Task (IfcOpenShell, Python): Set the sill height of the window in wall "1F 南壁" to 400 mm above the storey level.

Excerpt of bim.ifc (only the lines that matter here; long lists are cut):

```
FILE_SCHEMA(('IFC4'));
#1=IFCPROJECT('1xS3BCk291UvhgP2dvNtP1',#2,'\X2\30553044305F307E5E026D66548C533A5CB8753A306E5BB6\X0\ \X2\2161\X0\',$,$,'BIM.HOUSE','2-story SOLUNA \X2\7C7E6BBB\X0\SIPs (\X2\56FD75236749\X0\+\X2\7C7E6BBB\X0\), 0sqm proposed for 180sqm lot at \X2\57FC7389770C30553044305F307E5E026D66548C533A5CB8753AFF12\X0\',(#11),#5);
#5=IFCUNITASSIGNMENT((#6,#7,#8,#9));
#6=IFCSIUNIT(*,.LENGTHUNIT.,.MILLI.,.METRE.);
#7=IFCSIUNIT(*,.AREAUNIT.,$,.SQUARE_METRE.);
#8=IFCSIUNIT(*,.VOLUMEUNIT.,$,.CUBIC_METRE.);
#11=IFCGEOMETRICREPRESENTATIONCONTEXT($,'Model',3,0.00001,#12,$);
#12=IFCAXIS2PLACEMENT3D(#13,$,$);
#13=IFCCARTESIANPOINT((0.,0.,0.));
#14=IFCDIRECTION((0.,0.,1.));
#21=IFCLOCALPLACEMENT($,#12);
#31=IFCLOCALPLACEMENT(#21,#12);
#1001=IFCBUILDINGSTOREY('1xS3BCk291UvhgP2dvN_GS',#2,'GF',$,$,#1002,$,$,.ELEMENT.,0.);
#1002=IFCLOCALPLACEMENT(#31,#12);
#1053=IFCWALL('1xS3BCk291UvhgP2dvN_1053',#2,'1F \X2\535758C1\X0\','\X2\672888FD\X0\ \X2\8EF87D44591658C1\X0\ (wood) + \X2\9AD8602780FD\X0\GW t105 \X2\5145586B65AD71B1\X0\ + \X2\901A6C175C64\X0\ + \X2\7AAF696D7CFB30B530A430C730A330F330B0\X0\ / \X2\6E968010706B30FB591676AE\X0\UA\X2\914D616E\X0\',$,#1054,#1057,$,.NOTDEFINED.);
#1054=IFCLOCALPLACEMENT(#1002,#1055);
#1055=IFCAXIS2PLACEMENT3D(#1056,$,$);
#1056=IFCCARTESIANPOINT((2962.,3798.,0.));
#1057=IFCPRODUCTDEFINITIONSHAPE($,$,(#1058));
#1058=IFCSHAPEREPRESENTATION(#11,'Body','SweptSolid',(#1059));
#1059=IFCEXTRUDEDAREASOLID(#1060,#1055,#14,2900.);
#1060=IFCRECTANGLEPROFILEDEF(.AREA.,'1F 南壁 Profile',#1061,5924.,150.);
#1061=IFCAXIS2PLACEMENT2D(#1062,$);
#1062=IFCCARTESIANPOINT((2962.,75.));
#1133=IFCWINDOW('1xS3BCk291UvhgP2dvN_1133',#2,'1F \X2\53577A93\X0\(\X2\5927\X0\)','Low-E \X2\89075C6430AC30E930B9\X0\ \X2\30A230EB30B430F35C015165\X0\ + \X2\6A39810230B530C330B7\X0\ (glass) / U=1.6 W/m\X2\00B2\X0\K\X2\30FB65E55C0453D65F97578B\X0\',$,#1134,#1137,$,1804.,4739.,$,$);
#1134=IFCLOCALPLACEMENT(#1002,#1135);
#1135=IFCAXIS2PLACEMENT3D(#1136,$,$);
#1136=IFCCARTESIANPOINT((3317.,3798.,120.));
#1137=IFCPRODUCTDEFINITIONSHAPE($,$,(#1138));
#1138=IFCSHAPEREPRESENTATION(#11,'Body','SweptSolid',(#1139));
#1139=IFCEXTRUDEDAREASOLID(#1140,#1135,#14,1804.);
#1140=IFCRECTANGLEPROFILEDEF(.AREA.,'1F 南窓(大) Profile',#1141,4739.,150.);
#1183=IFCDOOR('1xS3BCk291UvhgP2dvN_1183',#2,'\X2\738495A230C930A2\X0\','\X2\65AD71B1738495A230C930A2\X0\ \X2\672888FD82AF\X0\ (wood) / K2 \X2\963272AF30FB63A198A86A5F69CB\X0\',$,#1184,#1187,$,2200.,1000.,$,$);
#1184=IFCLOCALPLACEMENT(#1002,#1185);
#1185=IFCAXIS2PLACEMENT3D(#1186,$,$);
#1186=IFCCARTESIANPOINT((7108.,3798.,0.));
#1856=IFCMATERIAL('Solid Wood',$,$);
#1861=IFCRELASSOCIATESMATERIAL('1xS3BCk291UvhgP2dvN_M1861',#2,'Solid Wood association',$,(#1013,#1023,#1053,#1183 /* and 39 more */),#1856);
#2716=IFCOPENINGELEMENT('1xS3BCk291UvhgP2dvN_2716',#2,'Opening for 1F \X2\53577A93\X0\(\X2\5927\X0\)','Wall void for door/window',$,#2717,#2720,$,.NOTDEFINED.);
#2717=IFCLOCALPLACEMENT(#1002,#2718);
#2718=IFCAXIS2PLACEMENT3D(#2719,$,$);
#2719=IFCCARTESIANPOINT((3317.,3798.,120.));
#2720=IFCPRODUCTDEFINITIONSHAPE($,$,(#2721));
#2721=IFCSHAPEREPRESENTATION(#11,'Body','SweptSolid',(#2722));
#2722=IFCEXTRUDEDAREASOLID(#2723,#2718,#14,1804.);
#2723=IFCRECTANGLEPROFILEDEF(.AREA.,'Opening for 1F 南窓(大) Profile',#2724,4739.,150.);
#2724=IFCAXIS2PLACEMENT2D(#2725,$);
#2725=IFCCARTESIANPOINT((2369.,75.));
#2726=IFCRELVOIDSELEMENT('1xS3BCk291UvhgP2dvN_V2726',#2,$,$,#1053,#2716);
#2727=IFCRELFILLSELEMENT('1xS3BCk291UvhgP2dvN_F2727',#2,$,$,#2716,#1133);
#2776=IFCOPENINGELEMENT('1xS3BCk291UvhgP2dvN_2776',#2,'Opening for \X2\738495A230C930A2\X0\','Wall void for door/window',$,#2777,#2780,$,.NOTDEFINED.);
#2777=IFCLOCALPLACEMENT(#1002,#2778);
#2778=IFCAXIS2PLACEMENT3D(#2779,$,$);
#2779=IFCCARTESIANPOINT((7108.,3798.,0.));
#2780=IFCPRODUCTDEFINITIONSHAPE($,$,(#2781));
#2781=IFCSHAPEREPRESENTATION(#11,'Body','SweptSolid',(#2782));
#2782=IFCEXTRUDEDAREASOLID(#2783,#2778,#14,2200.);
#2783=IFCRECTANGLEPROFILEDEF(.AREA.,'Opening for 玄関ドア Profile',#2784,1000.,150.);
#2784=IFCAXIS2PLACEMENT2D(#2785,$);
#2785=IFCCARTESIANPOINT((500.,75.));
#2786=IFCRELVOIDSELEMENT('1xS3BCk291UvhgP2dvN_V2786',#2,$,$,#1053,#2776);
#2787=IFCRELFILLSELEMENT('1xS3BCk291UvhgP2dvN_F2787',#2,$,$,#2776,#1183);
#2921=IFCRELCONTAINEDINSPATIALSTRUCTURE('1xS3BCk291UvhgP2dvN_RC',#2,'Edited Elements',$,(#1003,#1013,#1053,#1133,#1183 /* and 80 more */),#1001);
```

```python
import numpy as np
import ifcopenshell
import ifcopenshell.api.geometry
import ifcopenshell.geom
import ifcopenshell.util.element
import ifcopenshell.util.placement
import ifcopenshell.util.shape
import ifcopenshell.util.unit

model = ifcopenshell.open("bim.ifc")
unit_scale = ifcopenshell.util.unit.calculate_unit_scale(model)

window = model.by_id(1133)
opening = window.FillsVoids[0].RelatingOpeningElement
storey = ifcopenshell.util.element.get_container(window, ifc_class="IfcBuildingStorey")
level = ifcopenshell.util.placement.get_local_placement(storey.ObjectPlacement)[2, 3]

# The opening's origin need not be at the sill, so measure its lowest point.
shape = ifcopenshell.geom.create_shape(ifcopenshell.geom.settings(), opening)
bottom = ifcopenshell.util.shape.get_shape_bottom_elevation(shape, shape.geometry) / unit_scale
dz = level + 400.0 - bottom

shift = np.array([0.0, 0.0, dz])
# The window is not placed relative to its opening, so move both.
for product in (opening, window):
    matrix = ifcopenshell.util.placement.get_local_placement(product.ObjectPlacement)
    matrix[:3, 3] += shift
    ifcopenshell.api.geometry.edit_object_placement(model, product=product, matrix=matrix, is_si=False)

print(f"moved by {dz * unit_scale:+.3f} m")

model.write("bim_edited.ifc")
```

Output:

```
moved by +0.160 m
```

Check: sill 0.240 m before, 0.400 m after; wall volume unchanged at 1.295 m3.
